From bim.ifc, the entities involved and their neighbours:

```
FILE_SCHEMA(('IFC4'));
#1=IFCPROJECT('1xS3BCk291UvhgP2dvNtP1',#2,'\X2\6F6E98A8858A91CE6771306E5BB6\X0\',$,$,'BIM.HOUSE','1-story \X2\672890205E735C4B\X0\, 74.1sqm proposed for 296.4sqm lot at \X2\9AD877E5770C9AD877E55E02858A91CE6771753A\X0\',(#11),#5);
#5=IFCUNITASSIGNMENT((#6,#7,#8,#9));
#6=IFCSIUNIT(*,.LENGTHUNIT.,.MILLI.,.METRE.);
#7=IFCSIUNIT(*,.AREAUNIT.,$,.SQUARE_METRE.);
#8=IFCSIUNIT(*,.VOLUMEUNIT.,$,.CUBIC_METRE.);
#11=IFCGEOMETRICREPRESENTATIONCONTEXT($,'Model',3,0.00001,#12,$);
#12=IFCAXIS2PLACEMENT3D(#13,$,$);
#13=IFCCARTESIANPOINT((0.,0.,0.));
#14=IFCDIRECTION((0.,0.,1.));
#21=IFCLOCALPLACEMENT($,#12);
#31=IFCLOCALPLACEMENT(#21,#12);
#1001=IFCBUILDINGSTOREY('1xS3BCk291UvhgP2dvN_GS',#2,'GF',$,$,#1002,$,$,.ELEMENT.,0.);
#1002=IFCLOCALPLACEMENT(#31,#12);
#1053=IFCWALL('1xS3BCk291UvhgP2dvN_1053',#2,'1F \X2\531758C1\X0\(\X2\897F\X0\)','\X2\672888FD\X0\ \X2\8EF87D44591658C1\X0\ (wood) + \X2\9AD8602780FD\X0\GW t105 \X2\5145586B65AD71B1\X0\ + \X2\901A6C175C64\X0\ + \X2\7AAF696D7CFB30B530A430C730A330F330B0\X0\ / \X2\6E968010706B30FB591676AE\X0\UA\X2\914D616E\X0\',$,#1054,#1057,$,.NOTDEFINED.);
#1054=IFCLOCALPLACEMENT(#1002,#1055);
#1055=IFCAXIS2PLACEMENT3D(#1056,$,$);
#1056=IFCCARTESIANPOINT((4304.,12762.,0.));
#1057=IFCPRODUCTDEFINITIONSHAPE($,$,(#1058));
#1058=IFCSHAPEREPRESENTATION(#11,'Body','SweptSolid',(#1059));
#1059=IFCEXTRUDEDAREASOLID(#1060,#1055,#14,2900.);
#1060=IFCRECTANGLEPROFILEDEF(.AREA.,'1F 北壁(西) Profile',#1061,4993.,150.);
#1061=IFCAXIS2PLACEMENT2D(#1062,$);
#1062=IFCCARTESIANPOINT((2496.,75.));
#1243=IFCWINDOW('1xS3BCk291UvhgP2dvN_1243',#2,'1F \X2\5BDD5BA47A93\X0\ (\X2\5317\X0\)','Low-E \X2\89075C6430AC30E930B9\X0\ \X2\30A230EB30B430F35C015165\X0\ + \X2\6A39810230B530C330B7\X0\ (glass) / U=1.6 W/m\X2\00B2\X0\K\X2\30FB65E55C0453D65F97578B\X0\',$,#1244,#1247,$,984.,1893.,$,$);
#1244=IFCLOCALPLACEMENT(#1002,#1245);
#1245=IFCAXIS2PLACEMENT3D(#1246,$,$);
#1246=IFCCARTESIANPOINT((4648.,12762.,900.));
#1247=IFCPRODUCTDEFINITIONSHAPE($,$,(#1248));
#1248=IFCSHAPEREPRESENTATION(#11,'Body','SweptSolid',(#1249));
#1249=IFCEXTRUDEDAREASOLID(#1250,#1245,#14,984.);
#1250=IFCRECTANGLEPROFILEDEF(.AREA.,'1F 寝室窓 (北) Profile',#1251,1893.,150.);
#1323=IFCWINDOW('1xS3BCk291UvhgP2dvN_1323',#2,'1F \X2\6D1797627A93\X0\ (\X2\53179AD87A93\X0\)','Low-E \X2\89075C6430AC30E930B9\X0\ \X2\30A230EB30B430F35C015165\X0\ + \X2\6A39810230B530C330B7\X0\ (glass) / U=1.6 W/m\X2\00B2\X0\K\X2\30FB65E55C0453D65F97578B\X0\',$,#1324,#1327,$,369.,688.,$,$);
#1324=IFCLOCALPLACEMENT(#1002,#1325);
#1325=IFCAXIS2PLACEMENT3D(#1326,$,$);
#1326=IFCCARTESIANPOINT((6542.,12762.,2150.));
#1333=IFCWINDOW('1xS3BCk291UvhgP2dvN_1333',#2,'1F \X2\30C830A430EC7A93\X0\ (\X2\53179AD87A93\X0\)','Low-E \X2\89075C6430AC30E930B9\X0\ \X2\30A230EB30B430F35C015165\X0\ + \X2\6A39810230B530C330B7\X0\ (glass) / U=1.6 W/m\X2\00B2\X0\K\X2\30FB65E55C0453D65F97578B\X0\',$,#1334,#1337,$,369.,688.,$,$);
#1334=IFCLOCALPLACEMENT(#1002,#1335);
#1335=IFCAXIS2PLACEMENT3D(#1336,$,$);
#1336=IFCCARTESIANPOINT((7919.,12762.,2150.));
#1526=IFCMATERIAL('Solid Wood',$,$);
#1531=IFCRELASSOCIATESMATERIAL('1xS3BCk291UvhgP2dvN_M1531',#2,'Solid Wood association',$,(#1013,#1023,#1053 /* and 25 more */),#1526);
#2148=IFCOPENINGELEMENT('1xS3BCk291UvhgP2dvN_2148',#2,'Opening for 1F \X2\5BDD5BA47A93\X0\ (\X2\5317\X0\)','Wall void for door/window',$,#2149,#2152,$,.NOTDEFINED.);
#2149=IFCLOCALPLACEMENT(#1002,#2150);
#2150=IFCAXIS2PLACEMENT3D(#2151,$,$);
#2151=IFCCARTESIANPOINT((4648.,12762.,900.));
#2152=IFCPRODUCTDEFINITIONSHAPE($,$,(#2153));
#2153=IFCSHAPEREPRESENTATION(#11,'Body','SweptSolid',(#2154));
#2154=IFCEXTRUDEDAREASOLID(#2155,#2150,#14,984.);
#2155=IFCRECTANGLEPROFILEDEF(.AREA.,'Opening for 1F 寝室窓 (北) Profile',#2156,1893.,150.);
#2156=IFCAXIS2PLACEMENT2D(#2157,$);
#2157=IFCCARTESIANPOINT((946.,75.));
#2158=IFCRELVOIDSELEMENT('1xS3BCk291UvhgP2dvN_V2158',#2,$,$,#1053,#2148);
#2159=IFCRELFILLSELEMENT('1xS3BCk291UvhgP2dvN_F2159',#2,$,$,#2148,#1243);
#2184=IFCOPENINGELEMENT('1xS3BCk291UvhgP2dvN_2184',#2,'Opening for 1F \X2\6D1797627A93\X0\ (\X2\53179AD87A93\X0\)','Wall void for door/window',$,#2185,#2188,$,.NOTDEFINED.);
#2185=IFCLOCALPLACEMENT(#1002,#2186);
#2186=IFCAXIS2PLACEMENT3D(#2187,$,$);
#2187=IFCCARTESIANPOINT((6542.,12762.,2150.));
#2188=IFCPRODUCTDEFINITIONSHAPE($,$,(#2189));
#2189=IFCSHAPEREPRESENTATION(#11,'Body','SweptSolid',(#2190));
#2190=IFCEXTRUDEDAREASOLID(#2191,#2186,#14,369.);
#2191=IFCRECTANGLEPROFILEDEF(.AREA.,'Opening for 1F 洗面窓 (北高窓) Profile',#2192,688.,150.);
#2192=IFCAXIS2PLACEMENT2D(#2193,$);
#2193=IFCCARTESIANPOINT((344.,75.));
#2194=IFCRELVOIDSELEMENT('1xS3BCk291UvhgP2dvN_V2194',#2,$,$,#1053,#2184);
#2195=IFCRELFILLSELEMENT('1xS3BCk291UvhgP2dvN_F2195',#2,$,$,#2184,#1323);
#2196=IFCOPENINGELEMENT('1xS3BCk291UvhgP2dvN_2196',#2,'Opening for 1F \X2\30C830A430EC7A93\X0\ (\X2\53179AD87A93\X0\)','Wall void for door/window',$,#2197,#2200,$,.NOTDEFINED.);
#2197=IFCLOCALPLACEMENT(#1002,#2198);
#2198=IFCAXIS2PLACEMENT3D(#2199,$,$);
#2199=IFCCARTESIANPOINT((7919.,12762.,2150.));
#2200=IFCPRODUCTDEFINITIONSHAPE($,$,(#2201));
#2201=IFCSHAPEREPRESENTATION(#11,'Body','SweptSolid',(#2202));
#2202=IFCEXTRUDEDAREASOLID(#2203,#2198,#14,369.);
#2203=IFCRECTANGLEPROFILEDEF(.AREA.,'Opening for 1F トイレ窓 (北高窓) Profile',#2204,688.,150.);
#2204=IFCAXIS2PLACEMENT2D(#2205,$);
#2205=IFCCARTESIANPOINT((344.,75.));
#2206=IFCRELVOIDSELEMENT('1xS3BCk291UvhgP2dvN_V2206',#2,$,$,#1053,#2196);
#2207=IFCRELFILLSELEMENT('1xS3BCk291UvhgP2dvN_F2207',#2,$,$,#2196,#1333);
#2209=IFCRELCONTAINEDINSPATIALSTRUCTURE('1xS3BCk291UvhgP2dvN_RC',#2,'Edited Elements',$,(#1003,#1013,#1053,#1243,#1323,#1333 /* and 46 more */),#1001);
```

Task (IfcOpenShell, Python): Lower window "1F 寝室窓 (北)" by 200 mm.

```python
import numpy as np
import ifcopenshell
import ifcopenshell.api.geometry
import ifcopenshell.util.placement
import ifcopenshell.util.unit

model = ifcopenshell.open("bim.ifc")
unit_scale = ifcopenshell.util.unit.calculate_unit_scale(model)

window = model.by_guid("1xS3BCk291UvhgP2dvN_1243")
opening = window.FillsVoids[0].RelatingOpeningElement
dz = -200.0

shift = np.array([0.0, 0.0, dz])
# The window is not placed relative to its opening, so move both.
for product in (opening, window):
    matrix = ifcopenshell.util.placement.get_local_placement(product.ObjectPlacement)
    matrix[:3, 3] += shift
    ifcopenshell.api.geometry.edit_object_placement(model, product=product, matrix=matrix, is_si=False)

print(f"moved by {dz * unit_scale:+.3f} m")

model.write("bim_rev.ifc")
```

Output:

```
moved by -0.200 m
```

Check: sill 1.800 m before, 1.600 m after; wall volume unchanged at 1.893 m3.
